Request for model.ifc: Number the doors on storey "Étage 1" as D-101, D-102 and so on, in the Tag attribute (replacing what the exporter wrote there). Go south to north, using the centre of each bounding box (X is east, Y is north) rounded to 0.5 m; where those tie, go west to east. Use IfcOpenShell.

First a look at what the model holds.

```python
import ifcopenshell
import ifcopenshell.util.element
import ifcopenshell.util.placement

model = ifcopenshell.open("model.ifc")
print(model.schema)
storey = next(s for s in model.by_type("IfcBuildingStorey") if s.Name == "Étage 1")
doors = [e for e in ifcopenshell.util.element.get_decomposition(storey) if e.is_a("IfcDoor")]
for e in sorted(doors, key=lambda e: e.id()):
    origin = ifcopenshell.util.placement.get_local_placement(e.ObjectPlacement)[:3, 3]
    print(e.id(), e.Tag, e.Name, origin.round(2) + 0.0, sep=" | ")
```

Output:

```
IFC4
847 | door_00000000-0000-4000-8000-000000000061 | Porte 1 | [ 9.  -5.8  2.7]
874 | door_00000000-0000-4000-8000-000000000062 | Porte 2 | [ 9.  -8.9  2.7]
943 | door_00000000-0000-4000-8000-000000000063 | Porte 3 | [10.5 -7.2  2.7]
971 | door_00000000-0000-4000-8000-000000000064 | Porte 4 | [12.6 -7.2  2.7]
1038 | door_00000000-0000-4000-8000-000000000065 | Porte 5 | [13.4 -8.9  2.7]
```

```python
import ifcopenshell
import ifcopenshell.geom
import ifcopenshell.util.element
import ifcopenshell.util.shape

model = ifcopenshell.open("model.ifc")
settings = ifcopenshell.geom.settings()
settings.set("use-world-coords", True)


def centre(element):
    shape = ifcopenshell.geom.create_shape(settings, element)
    return ifcopenshell.util.shape.get_bbox_centroid(shape.geometry)


storey = next(s for s in model.by_type("IfcBuildingStorey") if s.Name == "Étage 1")
doors = [e for e in ifcopenshell.util.element.get_decomposition(storey) if e.is_a("IfcDoor")]

# Insertion points can sit at a corner or the storey origin, so sort by the geometry (in metres).
centres = {e: centre(e) for e in doors}
doors.sort(key=lambda e: (round(centres[e][1] / 0.5), centres[e][0]))

for i, e in enumerate(doors, start=1):
    number = f"D-1{i:02d}"
    e.Tag = number
    print(e.id(), number)

model.write("model_v2.ifc")
```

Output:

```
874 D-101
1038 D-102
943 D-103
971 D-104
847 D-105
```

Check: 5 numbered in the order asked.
